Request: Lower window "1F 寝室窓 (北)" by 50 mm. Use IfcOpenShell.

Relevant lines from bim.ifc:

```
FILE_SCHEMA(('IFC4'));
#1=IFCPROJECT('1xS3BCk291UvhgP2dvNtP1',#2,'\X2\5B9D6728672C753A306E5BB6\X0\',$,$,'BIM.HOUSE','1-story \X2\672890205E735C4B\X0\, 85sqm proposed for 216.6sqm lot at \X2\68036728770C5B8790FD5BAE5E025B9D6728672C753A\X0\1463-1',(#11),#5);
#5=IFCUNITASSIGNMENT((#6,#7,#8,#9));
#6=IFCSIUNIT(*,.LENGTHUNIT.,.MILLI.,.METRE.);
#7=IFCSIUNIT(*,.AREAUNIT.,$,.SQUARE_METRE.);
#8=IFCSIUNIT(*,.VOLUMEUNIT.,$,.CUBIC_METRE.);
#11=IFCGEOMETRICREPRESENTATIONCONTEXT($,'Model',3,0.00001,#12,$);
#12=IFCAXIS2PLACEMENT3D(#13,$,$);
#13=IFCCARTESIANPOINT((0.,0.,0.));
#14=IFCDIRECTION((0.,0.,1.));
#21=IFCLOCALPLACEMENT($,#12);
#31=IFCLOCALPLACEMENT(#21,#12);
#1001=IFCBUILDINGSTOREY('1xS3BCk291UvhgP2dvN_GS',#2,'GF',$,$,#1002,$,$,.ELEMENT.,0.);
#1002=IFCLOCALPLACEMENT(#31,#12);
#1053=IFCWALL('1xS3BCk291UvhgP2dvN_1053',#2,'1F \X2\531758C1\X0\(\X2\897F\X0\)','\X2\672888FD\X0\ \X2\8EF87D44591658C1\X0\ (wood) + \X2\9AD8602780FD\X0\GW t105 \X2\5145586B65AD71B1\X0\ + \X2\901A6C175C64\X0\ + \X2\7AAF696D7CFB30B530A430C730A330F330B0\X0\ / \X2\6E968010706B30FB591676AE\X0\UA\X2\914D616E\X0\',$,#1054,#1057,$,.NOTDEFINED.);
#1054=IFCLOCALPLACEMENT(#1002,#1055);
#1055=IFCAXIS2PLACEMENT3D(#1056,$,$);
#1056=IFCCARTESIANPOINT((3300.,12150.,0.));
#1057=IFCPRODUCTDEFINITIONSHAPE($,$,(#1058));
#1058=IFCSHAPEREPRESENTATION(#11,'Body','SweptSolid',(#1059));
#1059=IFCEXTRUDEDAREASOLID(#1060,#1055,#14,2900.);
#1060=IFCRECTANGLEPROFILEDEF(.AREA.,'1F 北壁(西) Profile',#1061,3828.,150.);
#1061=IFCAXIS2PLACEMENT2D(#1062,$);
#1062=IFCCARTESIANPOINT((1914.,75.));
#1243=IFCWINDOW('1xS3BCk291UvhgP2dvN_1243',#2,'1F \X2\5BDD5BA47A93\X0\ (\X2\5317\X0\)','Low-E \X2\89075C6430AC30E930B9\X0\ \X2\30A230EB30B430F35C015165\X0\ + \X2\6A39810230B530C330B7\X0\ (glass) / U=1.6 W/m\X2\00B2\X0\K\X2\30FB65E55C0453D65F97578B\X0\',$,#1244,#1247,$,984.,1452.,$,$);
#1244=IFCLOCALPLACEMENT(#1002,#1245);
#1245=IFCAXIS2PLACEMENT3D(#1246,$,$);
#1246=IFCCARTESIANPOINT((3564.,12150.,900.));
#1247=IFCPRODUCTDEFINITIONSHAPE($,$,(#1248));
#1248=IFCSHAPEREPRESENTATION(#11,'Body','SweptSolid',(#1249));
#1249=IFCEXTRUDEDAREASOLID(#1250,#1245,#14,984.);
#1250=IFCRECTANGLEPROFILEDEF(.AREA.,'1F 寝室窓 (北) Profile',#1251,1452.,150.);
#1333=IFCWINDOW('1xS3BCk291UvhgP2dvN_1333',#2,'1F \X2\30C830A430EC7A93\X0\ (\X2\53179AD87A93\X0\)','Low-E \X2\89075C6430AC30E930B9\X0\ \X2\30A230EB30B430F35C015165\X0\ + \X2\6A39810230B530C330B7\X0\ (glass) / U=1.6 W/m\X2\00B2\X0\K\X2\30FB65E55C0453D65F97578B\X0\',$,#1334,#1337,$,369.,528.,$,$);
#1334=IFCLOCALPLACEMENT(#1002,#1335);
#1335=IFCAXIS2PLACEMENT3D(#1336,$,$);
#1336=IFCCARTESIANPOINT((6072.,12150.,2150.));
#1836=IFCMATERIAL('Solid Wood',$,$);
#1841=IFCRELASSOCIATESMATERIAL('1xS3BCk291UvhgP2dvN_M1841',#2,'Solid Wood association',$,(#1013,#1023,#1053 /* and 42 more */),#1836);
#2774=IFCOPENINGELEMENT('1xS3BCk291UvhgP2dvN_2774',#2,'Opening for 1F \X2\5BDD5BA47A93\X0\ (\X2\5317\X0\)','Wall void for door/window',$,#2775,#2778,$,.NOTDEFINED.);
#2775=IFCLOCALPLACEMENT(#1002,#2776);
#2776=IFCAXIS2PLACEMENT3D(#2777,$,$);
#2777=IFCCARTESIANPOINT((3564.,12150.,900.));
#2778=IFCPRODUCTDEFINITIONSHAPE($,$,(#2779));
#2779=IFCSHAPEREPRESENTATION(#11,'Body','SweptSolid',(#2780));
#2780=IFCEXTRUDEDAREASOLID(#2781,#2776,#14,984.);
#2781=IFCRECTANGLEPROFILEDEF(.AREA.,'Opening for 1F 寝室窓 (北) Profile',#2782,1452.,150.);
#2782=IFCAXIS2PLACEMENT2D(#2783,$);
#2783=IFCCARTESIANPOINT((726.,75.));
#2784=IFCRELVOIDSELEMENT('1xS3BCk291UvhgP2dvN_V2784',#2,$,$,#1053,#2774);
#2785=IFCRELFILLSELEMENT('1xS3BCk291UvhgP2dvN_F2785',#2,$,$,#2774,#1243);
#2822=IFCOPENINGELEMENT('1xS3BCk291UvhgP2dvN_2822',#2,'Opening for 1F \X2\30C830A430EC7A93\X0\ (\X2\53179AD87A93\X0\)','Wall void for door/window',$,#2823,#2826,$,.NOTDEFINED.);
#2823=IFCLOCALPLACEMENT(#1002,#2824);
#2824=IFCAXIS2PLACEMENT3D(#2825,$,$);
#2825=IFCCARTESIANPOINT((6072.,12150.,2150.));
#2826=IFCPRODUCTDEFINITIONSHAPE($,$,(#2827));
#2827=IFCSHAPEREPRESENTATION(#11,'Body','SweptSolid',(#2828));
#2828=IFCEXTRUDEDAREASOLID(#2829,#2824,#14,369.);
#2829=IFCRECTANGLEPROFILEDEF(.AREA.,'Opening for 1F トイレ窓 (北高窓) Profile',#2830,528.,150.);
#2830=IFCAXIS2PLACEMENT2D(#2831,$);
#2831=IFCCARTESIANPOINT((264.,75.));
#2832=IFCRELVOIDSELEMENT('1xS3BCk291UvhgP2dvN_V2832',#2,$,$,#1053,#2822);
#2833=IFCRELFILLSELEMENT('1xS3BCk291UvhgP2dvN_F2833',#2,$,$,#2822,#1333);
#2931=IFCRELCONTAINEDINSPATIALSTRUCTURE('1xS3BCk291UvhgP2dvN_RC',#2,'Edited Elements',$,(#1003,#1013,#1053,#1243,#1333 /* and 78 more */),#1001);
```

```python
import numpy as np
import ifcopenshell
import ifcopenshell.api.geometry
import ifcopenshell.util.placement
import ifcopenshell.util.unit

model = ifcopenshell.open("bim.ifc")
unit_scale = ifcopenshell.util.unit.calculate_unit_scale(model)

window = model.by_guid("1xS3BCk291UvhgP2dvN_1243")
opening = window.FillsVoids[0].RelatingOpeningElement
dz = -0.05 / unit_scale

shift = np.array([0.0, 0.0, dz])
# The window is not placed relative to its opening, so move both.
for product in (opening, window):
    matrix = ifcopenshell.util.placement.get_local_placement(product.ObjectPlacement)
    matrix[:3, 3] += shift
    ifcopenshell.api.geometry.edit_object_placement(model, product=product, matrix=matrix, is_si=False)

print(f"moved by {dz * unit_scale:+.3f} m")

model.write("bim_updated.ifc")
```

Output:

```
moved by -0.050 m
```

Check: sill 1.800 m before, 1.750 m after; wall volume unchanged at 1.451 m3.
